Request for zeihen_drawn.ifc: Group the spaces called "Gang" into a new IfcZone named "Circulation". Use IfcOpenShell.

First a look at what the model holds.

```python
import ifcopenshell

model = ifcopenshell.open("zeihen_drawn.ifc")
print(model.schema)
seen = {}
for space in model.by_type("IfcSpace"):
    seen[space.LongName] = seen.get(space.LongName, 0) + 1
for name, count in sorted(seen.items(), key=str):
    print(count, "x", name)
print("zones:", [z.Name for z in model.by_type("IfcZone")][:20])
```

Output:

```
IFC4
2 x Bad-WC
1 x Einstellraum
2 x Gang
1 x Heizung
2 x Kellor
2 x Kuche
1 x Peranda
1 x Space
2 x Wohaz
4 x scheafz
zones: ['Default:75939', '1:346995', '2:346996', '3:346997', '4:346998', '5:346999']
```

```python
import ifcopenshell
import ifcopenshell.api.group
import ifcopenshell.api.root

model = ifcopenshell.open("zeihen_drawn.ifc")

names = {"Gang"}
spaces = [s for s in model.by_type("IfcSpace") if s.LongName in names]

zone = ifcopenshell.api.root.create_entity(model, ifc_class="IfcZone", name="Circulation")
ifcopenshell.api.group.assign_group(model, products=spaces, group=zone)
print(len(spaces), "spaces in", zone.Name)

model.write("zeihen_drawn_edited.ifc")
```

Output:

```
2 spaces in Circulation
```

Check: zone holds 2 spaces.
